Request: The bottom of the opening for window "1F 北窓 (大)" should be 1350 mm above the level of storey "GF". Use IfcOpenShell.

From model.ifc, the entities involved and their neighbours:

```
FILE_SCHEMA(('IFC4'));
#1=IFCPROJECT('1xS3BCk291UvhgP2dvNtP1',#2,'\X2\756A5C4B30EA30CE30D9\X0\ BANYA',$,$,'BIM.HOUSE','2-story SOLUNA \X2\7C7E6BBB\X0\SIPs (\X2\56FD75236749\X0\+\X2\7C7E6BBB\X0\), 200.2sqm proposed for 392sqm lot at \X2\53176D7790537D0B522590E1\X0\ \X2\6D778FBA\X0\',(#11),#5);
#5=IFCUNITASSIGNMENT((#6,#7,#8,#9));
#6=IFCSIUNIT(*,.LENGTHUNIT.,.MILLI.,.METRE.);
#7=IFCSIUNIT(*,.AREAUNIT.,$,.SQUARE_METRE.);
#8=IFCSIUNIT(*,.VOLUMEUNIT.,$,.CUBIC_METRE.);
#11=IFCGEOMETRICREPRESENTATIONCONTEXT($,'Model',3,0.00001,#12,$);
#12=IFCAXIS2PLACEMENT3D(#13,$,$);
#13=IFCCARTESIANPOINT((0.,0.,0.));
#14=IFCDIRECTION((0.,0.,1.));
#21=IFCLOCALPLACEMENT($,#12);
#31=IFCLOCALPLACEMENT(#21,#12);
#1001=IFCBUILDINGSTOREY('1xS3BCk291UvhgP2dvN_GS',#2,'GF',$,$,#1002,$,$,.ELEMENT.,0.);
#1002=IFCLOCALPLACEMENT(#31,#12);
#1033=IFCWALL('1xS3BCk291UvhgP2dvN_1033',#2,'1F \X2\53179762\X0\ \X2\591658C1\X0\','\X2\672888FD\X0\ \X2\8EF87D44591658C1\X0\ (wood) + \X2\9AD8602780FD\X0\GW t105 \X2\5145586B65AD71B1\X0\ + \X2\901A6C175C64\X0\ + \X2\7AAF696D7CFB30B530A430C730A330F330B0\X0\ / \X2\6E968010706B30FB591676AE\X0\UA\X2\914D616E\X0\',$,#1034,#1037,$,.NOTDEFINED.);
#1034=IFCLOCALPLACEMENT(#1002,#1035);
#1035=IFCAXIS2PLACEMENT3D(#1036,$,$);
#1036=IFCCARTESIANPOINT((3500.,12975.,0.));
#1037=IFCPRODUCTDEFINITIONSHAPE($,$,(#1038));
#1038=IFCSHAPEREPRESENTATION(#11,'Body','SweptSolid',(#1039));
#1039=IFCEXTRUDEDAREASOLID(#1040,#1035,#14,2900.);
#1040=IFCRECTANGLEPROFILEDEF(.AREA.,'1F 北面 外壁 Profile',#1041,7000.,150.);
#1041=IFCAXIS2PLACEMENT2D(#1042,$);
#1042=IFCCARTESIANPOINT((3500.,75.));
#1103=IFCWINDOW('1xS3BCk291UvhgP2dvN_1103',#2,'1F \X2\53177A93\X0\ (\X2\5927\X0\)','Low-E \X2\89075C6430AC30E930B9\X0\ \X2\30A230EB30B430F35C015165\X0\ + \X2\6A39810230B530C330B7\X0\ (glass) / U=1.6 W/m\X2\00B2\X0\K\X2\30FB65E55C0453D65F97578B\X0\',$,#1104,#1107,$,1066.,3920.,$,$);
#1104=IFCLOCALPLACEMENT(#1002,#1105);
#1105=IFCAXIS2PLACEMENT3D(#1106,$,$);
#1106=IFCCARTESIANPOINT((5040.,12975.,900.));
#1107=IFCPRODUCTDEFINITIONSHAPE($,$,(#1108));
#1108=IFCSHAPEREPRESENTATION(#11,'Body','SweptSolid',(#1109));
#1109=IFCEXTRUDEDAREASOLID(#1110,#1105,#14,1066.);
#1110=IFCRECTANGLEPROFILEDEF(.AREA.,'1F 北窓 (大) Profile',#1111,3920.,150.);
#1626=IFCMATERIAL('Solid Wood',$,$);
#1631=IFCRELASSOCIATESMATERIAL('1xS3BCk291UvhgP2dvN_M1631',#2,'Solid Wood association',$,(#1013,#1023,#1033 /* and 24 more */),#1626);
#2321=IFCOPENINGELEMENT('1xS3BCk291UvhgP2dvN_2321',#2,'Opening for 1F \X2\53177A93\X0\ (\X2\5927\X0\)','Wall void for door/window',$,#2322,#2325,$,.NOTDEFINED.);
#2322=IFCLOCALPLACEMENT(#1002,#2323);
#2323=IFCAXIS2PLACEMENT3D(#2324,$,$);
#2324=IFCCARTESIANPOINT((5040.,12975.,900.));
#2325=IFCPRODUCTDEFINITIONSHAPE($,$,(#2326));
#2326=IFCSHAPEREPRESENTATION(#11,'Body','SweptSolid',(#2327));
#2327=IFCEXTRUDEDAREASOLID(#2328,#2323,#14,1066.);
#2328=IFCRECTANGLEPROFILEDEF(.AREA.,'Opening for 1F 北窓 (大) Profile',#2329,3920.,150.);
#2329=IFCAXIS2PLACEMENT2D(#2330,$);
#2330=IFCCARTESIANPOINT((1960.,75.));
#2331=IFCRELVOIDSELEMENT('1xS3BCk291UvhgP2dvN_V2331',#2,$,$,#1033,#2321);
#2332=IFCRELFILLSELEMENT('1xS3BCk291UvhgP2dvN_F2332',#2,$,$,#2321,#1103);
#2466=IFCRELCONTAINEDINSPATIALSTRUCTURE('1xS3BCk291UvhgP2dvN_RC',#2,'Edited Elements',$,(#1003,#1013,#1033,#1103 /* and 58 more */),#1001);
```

```python
import numpy as np
import ifcopenshell
import ifcopenshell.api.geometry
import ifcopenshell.geom
import ifcopenshell.util.element
import ifcopenshell.util.placement
import ifcopenshell.util.shape
import ifcopenshell.util.unit

model = ifcopenshell.open("model.ifc")
unit_scale = ifcopenshell.util.unit.calculate_unit_scale(model)

window = model.by_id(1103)
opening = window.FillsVoids[0].RelatingOpeningElement
storey = ifcopenshell.util.element.get_container(window, ifc_class="IfcBuildingStorey")
level = ifcopenshell.util.placement.get_local_placement(storey.ObjectPlacement)[2, 3]

# The opening's origin need not be at the sill, so measure its lowest point.
shape = ifcopenshell.geom.create_shape(ifcopenshell.geom.settings(), opening)
bottom = ifcopenshell.util.shape.get_shape_bottom_elevation(shape, shape.geometry) / unit_scale
dz = level + 1.35 / unit_scale - bottom

shift = np.array([0.0, 0.0, dz])
# The window is not placed relative to its opening, so move both.
for product in (opening, window):
    matrix = ifcopenshell.util.placement.get_local_placement(product.ObjectPlacement)
    matrix[:3, 3] += shift
    ifcopenshell.api.geometry.edit_object_placement(model, product=product, matrix=matrix, is_si=False)

print(f"moved by {dz * unit_scale:+.3f} m")

model.write("model_rev.ifc")
```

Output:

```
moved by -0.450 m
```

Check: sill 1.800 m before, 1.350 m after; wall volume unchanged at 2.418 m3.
